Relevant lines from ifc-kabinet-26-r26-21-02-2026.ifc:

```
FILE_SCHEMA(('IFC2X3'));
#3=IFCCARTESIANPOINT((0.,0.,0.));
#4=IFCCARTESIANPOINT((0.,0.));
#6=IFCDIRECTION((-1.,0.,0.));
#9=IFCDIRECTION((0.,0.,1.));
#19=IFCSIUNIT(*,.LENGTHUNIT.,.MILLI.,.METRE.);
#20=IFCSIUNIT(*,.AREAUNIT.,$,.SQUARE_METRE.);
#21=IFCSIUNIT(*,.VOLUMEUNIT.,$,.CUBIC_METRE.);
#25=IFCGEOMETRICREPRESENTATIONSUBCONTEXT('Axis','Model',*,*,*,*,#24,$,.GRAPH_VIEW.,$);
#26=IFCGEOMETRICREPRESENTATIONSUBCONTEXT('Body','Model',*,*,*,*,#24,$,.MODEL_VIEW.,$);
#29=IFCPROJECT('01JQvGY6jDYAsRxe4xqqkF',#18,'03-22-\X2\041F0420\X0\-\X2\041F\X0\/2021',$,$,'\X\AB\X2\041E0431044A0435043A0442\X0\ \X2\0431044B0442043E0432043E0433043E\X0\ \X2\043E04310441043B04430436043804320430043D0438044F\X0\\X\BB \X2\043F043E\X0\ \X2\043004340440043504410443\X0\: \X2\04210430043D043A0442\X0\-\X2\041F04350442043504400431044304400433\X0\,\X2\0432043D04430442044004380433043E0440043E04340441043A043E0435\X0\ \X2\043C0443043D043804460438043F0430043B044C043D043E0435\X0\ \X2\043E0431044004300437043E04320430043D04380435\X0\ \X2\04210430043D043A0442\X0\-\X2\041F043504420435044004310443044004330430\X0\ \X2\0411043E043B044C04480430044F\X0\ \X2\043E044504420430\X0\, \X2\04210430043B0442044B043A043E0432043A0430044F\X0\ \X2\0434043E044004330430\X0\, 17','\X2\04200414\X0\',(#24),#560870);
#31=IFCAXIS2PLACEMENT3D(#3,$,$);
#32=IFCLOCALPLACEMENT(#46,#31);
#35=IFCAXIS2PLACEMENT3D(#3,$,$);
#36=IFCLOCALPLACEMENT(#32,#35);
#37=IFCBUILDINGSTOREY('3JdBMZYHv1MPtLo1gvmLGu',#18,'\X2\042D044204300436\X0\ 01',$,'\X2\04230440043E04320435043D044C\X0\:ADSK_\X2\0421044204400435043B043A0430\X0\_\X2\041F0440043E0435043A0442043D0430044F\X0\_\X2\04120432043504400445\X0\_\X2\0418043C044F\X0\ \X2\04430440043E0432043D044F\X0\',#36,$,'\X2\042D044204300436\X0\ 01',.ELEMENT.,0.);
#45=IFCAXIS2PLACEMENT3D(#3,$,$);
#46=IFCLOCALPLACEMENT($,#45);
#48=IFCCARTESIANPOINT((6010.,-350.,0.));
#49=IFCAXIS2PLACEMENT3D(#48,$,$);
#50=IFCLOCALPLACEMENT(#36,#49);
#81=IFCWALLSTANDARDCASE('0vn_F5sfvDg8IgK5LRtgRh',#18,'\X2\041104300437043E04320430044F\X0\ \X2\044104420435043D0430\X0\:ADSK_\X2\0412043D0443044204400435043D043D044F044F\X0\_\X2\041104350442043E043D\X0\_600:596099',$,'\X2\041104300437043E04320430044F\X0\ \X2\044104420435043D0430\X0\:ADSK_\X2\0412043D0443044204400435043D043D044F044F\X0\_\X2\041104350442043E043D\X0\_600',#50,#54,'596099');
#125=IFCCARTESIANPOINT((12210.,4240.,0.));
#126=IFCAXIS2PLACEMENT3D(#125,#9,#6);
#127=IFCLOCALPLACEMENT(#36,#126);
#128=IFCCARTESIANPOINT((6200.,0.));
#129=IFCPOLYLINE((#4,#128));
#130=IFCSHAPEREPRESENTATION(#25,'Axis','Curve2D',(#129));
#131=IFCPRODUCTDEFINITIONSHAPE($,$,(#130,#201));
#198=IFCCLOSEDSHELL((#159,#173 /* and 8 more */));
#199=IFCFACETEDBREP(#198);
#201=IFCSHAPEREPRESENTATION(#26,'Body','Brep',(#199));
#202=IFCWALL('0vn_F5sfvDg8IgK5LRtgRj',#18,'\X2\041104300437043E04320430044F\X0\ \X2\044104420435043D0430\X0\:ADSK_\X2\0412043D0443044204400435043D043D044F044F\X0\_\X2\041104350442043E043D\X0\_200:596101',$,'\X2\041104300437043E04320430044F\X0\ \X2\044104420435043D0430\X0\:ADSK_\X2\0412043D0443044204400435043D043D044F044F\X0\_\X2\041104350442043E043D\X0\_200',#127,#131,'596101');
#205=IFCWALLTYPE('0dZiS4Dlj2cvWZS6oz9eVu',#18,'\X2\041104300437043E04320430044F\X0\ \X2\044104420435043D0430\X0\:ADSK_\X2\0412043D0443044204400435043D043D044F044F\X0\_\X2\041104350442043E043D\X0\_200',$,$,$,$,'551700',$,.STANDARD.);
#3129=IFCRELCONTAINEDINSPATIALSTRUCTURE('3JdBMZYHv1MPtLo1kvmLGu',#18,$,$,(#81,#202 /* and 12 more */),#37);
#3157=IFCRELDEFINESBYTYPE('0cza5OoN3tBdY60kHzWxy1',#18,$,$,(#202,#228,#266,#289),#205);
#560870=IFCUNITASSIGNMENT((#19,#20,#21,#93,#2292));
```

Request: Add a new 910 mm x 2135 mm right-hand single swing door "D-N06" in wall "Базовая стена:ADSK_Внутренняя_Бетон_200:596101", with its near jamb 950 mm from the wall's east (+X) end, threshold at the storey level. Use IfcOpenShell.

```python
import numpy as np
import ifcopenshell
import ifcopenshell.api.feature
import ifcopenshell.api.geometry
import ifcopenshell.api.root
import ifcopenshell.api.spatial
import ifcopenshell.api.type
import ifcopenshell.geom
import ifcopenshell.util.element
import ifcopenshell.util.placement
import ifcopenshell.util.representation
import ifcopenshell.util.shape
import ifcopenshell.util.unit

model = ifcopenshell.open("ifc-kabinet-26-r26-21-02-2026.ifc")
unit_scale = ifcopenshell.util.unit.calculate_unit_scale(model)
settings = ifcopenshell.geom.settings()


def volume(element):
    """Net volume in cubic metres, openings subtracted."""
    shape = ifcopenshell.geom.create_shape(settings, element)
    return ifcopenshell.util.shape.get_volume(shape.geometry)


wall = model.by_guid("0vn_F5sfvDg8IgK5LRtgRj")
storey = ifcopenshell.util.element.get_container(wall, ifc_class="IfcBuildingStorey")
context = ifcopenshell.util.representation.get_context(model, "Model", "Body", "MODEL_VIEW")
before = volume(wall)

width, height, from_end, sill = 0.91, 2.135, 0.95, 0.0  # metres

# The wall runs along its own X axis, and the end named is its -X end.
wall_shape = ifcopenshell.geom.create_shape(settings, wall)
x, y, z = ifcopenshell.util.shape.get_vertices(wall_shape.geometry).T
start = x.min() + from_end
face, thickness = float(y.min()), float(y.max() - y.min())
wall_matrix = ifcopenshell.util.placement.get_local_placement(wall.ObjectPlacement)
level = ifcopenshell.util.placement.get_local_placement(storey.ObjectPlacement)[2, 3]


def in_wall(x, y):
    """Placement at x, y metres in the wall's axes, at sill height."""
    matrix = wall_matrix.copy()
    matrix[:, 3] = wall_matrix @ np.array([x / unit_scale, y / unit_scale, 0.0, 1.0])
    matrix[2, 3] = level + sill / unit_scale
    return matrix


# Opening: a box that overshoots both wall faces by 50 mm.
opening = ifcopenshell.api.root.create_entity(model, ifc_class="IfcOpeningElement")
box = ifcopenshell.api.geometry.add_wall_representation(
    model, context=context, length=width, height=height, thickness=thickness + 0.1
)
ifcopenshell.api.geometry.assign_representation(model, product=opening, representation=box)
ifcopenshell.api.geometry.edit_object_placement(model, product=opening, matrix=in_wall(start, face - 0.05), is_si=False)
ifcopenshell.api.feature.add_feature(model, feature=opening, element=wall)

door = ifcopenshell.api.root.create_entity(model, ifc_class="IfcDoor", name="D-N06")
door.OverallWidth, door.OverallHeight = width / unit_scale, height / unit_scale
body = ifcopenshell.api.geometry.add_door_representation(
    model,
    context=context,
    overall_width=door.OverallWidth,
    overall_height=door.OverallHeight,
    operation_type="SINGLE_SWING_RIGHT",
    lining_properties={"LiningDepth": thickness / unit_scale, "ThresholdDepth": thickness / unit_scale},
)
ifcopenshell.api.geometry.assign_representation(model, product=door, representation=body)
ifcopenshell.api.spatial.assign_container(model, products=[door], relating_structure=storey)
fills = ifcopenshell.api.feature.add_filling(model, opening=opening, element=door)
fills.OwnerHistory = door.OwnerHistory  # required in IFC2X3

# IFC2X3 keeps the operation on the door style.
style = ifcopenshell.api.root.create_entity(model, ifc_class="IfcDoorStyle", name="D-N06")
style.OperationType, style.ConstructionType = "SINGLE_SWING_RIGHT", "NOTDEFINED"
style.ParameterTakesPrecedence = style.Sizeable = False
ifcopenshell.api.type.assign_type(model, related_objects=[door], relating_type=style)

# The lining spans the wall, so the door starts at the wall face.
ifcopenshell.api.geometry.edit_object_placement(model, product=door, matrix=in_wall(start, face), is_si=False)

after = volume(wall)

print(f"wall volume {before:.3f} -> {after:.3f} m3")

model.write("ifc-kabinet-26-r26-21-02-2026_v2.ifc")
```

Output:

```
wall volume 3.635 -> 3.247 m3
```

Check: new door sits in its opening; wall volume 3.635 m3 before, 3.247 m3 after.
